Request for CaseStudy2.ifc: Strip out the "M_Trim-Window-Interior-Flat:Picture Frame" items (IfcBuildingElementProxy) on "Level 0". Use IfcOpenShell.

First a look at what the model holds.

```python
import ifcopenshell
import ifcopenshell.util.element

model = ifcopenshell.open("CaseStudy2.ifc")
print(model.schema)
storey = next(s for s in model.by_type("IfcBuildingStorey") if s.Name == "Level 0")
proxies = [e for e in ifcopenshell.util.element.get_decomposition(storey) if e.is_a("IfcBuildingElementProxy")]
seen = {}
for e in proxies:
    element_type = ifcopenshell.util.element.get_type(e)
    name = element_type.Name if element_type not in (None, e) else None
    seen[name] = seen.get(name, 0) + 1
for name, count in sorted(seen.items(), key=str):
    print(count, "x", name)
```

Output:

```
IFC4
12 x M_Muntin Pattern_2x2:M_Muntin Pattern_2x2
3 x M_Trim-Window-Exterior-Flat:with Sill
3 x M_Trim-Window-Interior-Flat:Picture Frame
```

```python
import ifcopenshell
import ifcopenshell.api.root
import ifcopenshell.util.element

model = ifcopenshell.open("CaseStudy2.ifc")

storey = next(s for s in model.by_type("IfcBuildingStorey") if s.Name == "Level 0")
proxies = [e for e in ifcopenshell.util.element.get_decomposition(storey) if e.is_a("IfcBuildingElementProxy")]
targets = [e for e in proxies if (t := ifcopenshell.util.element.get_type(e)) not in (None, e) and t.Name == "M_Trim-Window-Interior-Flat:Picture Frame"]

for e in targets:
    ifcopenshell.api.root.remove_product(model, product=e)
print(len(targets), "removed")

model.write("CaseStudy2_updated.ifc")
```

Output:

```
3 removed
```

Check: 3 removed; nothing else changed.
